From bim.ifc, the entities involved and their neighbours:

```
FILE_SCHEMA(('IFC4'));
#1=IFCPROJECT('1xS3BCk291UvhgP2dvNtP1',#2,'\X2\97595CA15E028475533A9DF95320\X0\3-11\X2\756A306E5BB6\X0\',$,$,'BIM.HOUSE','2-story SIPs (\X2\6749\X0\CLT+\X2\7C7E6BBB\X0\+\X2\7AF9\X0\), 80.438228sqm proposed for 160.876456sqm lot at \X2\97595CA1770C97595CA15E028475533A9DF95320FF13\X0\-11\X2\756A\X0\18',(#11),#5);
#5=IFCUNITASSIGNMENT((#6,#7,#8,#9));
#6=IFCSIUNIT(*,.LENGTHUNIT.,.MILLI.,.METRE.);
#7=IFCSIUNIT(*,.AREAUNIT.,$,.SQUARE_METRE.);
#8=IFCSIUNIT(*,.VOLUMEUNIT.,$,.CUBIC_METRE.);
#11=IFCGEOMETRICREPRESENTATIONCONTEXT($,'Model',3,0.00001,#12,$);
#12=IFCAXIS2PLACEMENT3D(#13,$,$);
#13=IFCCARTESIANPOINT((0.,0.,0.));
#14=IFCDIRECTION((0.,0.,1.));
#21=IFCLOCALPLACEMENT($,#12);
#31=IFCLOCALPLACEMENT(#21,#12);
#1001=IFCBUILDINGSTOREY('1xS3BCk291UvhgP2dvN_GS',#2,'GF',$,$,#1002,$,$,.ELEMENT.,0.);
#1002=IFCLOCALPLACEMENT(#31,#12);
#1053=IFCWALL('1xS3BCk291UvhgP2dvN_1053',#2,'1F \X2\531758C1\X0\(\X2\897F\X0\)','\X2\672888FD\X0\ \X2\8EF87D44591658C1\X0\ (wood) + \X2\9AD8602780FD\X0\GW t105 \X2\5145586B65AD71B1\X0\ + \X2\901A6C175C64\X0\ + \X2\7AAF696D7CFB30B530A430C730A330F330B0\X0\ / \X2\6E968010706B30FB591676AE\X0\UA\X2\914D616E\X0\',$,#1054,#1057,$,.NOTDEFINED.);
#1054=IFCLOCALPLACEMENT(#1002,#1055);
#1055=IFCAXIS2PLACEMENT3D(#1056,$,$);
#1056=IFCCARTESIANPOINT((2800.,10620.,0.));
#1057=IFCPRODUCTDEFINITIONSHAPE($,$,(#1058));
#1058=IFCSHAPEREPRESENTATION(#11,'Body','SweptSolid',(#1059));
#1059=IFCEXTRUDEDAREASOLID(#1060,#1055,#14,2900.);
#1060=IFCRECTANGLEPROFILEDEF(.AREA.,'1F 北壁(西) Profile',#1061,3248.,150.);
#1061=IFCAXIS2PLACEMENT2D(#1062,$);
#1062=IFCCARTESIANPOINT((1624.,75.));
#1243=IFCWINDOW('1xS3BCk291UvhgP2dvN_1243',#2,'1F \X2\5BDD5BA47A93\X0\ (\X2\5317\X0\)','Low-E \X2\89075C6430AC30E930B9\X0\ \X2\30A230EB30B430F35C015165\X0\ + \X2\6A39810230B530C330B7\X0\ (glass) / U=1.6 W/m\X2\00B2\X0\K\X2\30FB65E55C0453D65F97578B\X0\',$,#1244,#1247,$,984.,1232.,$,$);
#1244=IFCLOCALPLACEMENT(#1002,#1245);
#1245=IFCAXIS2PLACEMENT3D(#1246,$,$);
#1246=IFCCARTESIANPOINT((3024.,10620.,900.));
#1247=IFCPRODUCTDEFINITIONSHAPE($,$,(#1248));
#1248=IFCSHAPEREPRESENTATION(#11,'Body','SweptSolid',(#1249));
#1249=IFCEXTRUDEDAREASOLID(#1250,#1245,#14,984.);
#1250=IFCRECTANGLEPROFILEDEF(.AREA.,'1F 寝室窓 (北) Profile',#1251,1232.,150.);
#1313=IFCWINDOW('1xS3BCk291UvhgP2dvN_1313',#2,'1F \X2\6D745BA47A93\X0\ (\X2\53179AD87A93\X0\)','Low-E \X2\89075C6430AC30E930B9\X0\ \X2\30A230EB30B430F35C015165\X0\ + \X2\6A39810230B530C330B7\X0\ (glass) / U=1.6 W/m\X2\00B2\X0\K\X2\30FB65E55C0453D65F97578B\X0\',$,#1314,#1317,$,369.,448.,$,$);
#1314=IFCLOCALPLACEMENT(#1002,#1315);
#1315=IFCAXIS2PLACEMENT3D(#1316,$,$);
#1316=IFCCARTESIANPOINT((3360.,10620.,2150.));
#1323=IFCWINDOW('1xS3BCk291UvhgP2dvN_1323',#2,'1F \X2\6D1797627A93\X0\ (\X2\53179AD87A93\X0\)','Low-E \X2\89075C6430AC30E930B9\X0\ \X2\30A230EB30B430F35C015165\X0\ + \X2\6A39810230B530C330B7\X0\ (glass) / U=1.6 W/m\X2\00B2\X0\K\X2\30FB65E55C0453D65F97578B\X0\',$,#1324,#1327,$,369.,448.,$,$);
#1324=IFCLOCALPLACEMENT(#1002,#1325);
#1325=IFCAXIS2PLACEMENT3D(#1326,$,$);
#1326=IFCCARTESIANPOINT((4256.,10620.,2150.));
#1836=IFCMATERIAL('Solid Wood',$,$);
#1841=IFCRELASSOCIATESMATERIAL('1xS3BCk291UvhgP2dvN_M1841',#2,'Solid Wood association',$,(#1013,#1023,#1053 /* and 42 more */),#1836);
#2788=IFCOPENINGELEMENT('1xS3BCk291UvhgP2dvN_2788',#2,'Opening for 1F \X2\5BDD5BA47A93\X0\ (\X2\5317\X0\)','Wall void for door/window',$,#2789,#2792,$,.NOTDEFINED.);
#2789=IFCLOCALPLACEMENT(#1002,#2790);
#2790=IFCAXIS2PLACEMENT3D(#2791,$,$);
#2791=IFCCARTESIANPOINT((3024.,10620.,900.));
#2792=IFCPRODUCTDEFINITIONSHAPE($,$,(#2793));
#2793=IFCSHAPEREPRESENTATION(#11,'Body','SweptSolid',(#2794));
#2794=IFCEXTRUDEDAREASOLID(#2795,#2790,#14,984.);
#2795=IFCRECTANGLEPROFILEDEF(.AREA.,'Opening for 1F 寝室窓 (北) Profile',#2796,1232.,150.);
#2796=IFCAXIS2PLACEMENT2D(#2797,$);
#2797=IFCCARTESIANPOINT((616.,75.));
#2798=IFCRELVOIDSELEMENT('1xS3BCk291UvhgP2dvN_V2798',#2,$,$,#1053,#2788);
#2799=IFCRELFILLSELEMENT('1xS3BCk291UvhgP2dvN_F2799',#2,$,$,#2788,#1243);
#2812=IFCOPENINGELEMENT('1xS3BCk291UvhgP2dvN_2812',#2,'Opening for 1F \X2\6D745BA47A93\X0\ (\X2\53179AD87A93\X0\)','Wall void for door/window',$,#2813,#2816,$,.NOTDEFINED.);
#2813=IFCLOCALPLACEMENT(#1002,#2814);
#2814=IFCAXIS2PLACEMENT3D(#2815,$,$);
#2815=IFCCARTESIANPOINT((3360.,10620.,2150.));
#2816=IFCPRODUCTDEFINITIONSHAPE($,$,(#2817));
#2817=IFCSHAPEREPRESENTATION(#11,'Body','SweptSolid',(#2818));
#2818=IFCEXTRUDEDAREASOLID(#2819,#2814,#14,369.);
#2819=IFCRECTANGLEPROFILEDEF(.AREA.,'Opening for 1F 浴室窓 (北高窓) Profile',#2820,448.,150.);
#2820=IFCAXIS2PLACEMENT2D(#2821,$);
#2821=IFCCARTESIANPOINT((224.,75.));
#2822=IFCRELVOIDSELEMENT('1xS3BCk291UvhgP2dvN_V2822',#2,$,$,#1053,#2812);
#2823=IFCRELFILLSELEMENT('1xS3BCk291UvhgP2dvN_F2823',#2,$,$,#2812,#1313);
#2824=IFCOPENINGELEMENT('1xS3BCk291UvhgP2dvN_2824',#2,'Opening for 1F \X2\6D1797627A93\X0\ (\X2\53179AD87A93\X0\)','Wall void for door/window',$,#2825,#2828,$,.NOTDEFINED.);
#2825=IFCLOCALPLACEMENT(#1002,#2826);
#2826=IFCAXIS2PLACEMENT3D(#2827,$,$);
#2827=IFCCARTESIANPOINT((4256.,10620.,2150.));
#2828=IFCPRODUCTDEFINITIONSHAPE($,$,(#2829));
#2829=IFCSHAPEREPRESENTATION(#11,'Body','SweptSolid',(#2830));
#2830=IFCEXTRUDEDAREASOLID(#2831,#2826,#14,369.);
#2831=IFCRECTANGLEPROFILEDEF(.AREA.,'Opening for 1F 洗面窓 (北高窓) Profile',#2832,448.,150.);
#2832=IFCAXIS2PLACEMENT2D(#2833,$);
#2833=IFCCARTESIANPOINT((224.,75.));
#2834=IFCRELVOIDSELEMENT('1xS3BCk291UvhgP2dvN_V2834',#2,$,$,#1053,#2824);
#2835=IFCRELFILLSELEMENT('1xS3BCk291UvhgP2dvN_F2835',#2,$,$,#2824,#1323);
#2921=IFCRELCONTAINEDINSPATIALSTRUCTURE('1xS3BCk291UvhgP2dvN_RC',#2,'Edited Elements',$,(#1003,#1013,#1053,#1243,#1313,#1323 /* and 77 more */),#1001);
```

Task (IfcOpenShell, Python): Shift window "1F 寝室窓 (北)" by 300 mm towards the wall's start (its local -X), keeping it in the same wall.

```python
import ifcopenshell
import ifcopenshell.api.geometry
import ifcopenshell.util.placement

model = ifcopenshell.open("bim.ifc")

window = model.by_guid("1xS3BCk291UvhgP2dvN_1243")
opening = window.FillsVoids[0].RelatingOpeningElement
wall = opening.VoidsElements[0].RelatingBuildingElement

wall_matrix = ifcopenshell.util.placement.get_local_placement(wall.ObjectPlacement)
shift = wall_matrix[:3, 0] * -300.0
before = ifcopenshell.util.placement.get_local_placement(window.ObjectPlacement)[:3, 3].copy()

# The window is not placed relative to its opening, so move both.
for product in (opening, window):
    matrix = ifcopenshell.util.placement.get_local_placement(product.ObjectPlacement)
    matrix[:3, 3] += shift
    ifcopenshell.api.geometry.edit_object_placement(model, product=product, matrix=matrix, is_si=False)

after = ifcopenshell.util.placement.get_local_placement(window.ObjectPlacement)[:3, 3]
print("window moved by", (after - before).round(3) + 0.0)

model.write("bim_rev.ifc")
```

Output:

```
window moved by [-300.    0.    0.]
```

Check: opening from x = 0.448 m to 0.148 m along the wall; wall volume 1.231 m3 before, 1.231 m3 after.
